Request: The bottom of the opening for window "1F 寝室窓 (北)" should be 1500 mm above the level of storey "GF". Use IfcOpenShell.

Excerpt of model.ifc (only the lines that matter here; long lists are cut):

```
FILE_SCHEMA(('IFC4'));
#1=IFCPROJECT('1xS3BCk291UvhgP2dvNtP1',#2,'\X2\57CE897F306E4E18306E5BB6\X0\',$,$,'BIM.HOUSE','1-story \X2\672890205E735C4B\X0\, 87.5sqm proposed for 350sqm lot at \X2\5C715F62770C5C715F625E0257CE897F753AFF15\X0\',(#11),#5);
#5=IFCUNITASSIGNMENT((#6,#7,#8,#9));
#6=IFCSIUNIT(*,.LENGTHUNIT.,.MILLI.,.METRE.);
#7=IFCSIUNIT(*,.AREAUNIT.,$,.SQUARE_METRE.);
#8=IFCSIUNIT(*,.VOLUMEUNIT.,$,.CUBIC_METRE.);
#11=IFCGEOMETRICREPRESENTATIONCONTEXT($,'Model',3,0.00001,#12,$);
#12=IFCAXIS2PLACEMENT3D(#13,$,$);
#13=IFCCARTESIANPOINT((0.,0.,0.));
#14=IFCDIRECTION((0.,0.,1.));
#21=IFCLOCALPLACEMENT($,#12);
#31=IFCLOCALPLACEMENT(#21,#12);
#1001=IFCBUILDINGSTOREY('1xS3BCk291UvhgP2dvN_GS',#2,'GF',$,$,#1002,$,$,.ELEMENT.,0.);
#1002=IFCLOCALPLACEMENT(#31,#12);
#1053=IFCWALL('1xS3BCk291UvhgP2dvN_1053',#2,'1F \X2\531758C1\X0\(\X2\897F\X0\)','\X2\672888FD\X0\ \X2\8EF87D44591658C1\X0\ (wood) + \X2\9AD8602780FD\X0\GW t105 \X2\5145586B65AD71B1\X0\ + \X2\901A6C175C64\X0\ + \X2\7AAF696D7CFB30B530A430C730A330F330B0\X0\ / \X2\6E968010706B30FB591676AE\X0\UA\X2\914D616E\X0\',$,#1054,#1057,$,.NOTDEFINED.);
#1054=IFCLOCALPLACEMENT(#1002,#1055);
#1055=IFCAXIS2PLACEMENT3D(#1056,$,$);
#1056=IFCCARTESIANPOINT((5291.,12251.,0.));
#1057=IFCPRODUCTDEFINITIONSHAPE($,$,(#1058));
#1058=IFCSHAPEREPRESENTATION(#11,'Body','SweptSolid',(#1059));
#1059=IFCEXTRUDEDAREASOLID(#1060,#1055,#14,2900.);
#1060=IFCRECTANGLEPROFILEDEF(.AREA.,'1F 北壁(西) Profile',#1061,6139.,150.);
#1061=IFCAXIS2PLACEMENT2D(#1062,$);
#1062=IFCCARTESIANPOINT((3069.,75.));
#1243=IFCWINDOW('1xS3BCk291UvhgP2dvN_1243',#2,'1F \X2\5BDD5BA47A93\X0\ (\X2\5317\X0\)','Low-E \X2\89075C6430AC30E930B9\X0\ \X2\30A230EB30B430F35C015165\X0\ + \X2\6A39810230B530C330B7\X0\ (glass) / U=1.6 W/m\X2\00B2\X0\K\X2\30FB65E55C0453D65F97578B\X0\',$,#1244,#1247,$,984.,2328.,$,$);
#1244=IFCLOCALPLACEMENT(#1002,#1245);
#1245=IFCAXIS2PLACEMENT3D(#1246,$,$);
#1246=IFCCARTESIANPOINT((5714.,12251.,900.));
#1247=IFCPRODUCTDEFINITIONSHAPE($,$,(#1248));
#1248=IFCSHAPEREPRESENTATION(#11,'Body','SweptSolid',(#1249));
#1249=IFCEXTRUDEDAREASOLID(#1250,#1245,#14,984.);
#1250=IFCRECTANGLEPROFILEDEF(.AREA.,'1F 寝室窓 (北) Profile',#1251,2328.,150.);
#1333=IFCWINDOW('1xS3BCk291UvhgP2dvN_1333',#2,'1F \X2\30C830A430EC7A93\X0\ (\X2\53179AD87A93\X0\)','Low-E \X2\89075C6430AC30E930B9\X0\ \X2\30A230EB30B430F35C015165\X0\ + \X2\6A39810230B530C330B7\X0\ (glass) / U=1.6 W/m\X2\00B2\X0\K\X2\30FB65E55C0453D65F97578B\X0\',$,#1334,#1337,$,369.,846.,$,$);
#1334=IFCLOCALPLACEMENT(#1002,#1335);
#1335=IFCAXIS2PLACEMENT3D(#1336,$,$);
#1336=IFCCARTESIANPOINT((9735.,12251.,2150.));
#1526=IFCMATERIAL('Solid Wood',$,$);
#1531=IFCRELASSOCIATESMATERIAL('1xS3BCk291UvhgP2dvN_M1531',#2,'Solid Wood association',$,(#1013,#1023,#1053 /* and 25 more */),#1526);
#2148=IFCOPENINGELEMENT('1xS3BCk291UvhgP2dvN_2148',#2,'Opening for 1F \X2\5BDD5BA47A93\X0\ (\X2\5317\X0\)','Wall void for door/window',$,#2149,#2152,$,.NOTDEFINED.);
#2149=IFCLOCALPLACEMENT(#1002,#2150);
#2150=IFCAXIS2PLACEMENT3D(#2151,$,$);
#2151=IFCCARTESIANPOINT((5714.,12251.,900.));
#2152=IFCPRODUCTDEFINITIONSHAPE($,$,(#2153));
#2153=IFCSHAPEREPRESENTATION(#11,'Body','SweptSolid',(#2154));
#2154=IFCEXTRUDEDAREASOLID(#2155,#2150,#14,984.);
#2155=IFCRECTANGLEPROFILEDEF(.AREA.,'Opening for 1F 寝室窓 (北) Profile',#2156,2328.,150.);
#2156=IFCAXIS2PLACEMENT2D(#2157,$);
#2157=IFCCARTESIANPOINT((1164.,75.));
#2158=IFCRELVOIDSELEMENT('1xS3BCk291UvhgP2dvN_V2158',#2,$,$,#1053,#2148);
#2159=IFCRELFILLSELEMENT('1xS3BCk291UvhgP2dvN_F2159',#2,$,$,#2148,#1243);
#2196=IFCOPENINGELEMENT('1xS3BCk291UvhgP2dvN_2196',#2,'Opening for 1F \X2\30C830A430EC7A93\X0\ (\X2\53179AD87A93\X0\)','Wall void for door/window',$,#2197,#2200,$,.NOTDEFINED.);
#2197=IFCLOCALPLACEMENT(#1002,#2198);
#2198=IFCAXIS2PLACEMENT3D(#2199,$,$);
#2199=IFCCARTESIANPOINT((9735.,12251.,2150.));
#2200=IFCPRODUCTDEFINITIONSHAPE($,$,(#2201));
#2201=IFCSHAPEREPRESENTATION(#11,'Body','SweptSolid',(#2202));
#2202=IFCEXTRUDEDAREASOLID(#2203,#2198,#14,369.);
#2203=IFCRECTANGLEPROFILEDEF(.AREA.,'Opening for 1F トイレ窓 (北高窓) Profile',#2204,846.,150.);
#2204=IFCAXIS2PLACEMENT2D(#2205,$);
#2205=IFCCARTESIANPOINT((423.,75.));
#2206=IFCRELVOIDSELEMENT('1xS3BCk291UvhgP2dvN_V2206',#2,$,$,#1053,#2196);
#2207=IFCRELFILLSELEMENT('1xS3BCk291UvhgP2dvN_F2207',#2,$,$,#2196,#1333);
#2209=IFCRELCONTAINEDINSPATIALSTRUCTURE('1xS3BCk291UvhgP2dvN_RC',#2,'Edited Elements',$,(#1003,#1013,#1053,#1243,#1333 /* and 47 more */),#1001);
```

```python
import numpy as np
import ifcopenshell
import ifcopenshell.api.geometry
import ifcopenshell.geom
import ifcopenshell.util.element
import ifcopenshell.util.placement
import ifcopenshell.util.shape
import ifcopenshell.util.unit

model = ifcopenshell.open("model.ifc")
unit_scale = ifcopenshell.util.unit.calculate_unit_scale(model)

window = model.by_guid("1xS3BCk291UvhgP2dvN_1243")
opening = window.FillsVoids[0].RelatingOpeningElement
storey = ifcopenshell.util.element.get_container(window, ifc_class="IfcBuildingStorey")
level = ifcopenshell.util.placement.get_local_placement(storey.ObjectPlacement)[2, 3]

# The opening's origin need not be at the sill, so measure its lowest point.
shape = ifcopenshell.geom.create_shape(ifcopenshell.geom.settings(), opening)
bottom = ifcopenshell.util.shape.get_shape_bottom_elevation(shape, shape.geometry) / unit_scale
dz = level + 1.5 / unit_scale - bottom

shift = np.array([0.0, 0.0, dz])
# The window is not placed relative to its opening, so move both.
for product in (opening, window):
    matrix = ifcopenshell.util.placement.get_local_placement(product.ObjectPlacement)
    matrix[:3, 3] += shift
    ifcopenshell.api.geometry.edit_object_placement(model, product=product, matrix=matrix, is_si=False)

print(f"moved by {dz * unit_scale:+.3f} m")

model.write("model_rev.ifc")
```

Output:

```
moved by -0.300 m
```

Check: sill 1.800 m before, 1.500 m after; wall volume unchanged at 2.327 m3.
